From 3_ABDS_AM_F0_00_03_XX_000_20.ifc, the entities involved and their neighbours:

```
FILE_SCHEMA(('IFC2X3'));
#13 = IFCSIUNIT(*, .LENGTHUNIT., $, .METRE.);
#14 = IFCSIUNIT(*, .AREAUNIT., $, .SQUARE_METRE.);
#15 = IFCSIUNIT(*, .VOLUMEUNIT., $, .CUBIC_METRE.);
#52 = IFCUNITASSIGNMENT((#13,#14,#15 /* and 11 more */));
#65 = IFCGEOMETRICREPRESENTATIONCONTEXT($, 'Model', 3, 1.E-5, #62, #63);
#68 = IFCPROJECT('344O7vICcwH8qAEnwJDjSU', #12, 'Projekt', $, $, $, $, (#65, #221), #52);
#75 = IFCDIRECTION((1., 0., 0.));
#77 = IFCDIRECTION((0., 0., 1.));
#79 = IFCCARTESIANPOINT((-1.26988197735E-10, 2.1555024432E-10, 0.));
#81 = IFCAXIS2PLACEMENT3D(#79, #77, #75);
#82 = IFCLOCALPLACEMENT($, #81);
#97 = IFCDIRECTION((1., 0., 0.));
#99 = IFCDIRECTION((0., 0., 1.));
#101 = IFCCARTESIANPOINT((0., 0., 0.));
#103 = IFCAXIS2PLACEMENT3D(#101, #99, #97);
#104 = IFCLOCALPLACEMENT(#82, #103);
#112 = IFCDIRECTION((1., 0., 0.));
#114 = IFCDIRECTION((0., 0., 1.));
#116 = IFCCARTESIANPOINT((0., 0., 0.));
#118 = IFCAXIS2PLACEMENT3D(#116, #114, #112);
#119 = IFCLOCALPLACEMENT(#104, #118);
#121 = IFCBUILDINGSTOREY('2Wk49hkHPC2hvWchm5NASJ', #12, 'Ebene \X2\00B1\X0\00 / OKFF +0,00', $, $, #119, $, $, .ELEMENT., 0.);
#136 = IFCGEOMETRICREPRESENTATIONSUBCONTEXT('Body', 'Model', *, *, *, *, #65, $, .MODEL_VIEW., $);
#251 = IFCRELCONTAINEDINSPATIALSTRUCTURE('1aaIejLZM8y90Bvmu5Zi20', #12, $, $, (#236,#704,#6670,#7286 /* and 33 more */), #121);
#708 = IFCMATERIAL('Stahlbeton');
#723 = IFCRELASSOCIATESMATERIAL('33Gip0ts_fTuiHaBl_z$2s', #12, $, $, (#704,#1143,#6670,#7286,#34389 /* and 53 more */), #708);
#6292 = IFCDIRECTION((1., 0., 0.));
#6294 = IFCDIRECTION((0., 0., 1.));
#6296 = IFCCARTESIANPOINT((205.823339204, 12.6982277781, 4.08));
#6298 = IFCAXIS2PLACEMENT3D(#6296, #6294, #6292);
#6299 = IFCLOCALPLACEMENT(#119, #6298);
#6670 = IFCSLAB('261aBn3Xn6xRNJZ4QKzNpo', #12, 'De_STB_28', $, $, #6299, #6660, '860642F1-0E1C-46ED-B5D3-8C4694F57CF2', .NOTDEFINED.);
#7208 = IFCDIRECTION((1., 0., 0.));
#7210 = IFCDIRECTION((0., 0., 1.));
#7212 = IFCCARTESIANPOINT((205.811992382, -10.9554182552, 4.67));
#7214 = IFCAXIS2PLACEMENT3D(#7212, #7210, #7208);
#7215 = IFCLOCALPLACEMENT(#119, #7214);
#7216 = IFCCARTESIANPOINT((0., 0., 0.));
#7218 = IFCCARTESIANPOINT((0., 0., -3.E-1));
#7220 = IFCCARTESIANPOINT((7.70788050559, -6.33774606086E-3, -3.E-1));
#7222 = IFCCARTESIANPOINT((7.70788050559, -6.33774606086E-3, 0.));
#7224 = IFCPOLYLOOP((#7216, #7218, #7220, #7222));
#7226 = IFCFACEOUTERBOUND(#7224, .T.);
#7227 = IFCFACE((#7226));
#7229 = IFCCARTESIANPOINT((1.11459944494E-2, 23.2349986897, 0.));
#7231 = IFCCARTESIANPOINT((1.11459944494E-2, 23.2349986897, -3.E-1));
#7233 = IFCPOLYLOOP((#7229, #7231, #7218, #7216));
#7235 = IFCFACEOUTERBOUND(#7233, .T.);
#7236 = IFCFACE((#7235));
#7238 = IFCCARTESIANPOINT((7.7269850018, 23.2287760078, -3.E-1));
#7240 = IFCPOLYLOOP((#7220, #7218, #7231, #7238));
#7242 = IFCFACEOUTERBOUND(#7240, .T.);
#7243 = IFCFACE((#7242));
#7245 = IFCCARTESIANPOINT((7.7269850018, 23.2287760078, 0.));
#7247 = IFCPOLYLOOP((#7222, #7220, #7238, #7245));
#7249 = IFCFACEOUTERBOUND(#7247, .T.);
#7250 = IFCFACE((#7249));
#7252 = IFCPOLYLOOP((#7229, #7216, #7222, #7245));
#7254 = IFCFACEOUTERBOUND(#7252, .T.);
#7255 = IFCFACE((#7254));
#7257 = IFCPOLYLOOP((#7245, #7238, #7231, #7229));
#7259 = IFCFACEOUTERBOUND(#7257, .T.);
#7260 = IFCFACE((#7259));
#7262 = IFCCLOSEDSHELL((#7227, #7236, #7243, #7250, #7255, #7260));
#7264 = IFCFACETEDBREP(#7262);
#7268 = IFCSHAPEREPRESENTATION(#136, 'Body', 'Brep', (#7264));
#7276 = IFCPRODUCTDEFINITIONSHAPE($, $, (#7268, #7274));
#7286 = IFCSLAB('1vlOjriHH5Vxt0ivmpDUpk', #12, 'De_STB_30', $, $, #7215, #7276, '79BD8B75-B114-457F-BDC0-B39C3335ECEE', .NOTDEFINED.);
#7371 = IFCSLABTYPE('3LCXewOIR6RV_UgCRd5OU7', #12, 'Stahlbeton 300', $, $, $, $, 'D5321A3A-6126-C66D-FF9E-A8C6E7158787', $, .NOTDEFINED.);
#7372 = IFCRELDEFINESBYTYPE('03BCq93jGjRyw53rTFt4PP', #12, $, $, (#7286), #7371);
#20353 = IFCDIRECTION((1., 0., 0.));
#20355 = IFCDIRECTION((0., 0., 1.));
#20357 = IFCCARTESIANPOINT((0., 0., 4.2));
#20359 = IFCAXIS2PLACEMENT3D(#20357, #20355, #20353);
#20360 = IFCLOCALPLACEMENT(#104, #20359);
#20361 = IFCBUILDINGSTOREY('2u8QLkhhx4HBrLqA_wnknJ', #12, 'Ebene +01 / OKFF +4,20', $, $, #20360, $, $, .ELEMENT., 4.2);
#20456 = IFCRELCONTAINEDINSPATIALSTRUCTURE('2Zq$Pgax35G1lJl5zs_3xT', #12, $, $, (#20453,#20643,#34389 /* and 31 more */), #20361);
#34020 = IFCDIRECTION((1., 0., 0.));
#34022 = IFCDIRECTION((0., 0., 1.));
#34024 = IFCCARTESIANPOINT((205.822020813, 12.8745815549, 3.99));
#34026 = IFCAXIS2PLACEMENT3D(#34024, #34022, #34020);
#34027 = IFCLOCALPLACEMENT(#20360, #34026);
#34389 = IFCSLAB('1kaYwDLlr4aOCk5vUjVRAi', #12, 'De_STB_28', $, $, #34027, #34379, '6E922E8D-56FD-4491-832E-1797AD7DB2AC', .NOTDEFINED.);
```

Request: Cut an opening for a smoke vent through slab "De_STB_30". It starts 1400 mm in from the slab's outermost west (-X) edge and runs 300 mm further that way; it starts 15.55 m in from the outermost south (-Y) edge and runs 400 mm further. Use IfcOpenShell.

```python
import numpy as np
import ifcopenshell
import ifcopenshell.api.feature
import ifcopenshell.api.geometry
import ifcopenshell.api.root
import ifcopenshell.geom
import ifcopenshell.util.placement
import ifcopenshell.util.representation
import ifcopenshell.util.shape
import ifcopenshell.util.unit

model = ifcopenshell.open("3_ABDS_AM_F0_00_03_XX_000_20.ifc")
unit_scale = ifcopenshell.util.unit.calculate_unit_scale(model)
settings = ifcopenshell.geom.settings()


def volume(element):
    """Net volume in cubic metres, openings subtracted."""
    shape = ifcopenshell.geom.create_shape(settings, element)
    return ifcopenshell.util.shape.get_volume(shape.geometry)


slab = model.by_guid("1vlOjriHH5Vxt0ivmpDUpk")
before = volume(slab)

# Extent in the slab's own axes, in metres. The edges named are its -X and -Y sides.
slab_shape = ifcopenshell.geom.create_shape(settings, slab)
vertices = ifcopenshell.util.shape.get_vertices(slab_shape.geometry)
x_min, y_min, bottom = vertices.min(axis=0)
top = vertices[:, 2].max()

opening = ifcopenshell.api.root.create_entity(model, ifc_class="IfcOpeningElement", name="Smoke vent opening")
context = ifcopenshell.util.representation.get_context(model, "Model", "Body", "MODEL_VIEW")
width, depth = 0.3, 0.4
outline = [(0.0, 0.0), (width, 0.0), (width, depth), (0.0, depth), (0.0, 0.0)]
# Overshoot both faces by 50 mm so the cut is clean.
shape = ifcopenshell.api.geometry.add_slab_representation(
    model, context=context, depth=top - bottom + 0.1, polyline=outline
)
ifcopenshell.api.geometry.assign_representation(model, product=opening, representation=shape)

matrix = ifcopenshell.util.placement.get_local_placement(slab.ObjectPlacement)
matrix[:, 3] = matrix @ np.append(np.array([x_min + 1.4, y_min + 15.55, bottom - 0.05]) / unit_scale, 1.0)
ifcopenshell.api.geometry.edit_object_placement(model, product=opening, matrix=matrix, is_si=False)
ifcopenshell.api.feature.add_feature(model, feature=opening, element=slab)

after = volume(slab)

print(f"slab volume {before:.3f} -> {after:.3f} m3")

model.write("3_ABDS_AM_F0_00_03_XX_000_20_updated.ifc")
```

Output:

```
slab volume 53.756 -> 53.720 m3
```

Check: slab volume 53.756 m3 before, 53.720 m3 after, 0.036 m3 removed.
